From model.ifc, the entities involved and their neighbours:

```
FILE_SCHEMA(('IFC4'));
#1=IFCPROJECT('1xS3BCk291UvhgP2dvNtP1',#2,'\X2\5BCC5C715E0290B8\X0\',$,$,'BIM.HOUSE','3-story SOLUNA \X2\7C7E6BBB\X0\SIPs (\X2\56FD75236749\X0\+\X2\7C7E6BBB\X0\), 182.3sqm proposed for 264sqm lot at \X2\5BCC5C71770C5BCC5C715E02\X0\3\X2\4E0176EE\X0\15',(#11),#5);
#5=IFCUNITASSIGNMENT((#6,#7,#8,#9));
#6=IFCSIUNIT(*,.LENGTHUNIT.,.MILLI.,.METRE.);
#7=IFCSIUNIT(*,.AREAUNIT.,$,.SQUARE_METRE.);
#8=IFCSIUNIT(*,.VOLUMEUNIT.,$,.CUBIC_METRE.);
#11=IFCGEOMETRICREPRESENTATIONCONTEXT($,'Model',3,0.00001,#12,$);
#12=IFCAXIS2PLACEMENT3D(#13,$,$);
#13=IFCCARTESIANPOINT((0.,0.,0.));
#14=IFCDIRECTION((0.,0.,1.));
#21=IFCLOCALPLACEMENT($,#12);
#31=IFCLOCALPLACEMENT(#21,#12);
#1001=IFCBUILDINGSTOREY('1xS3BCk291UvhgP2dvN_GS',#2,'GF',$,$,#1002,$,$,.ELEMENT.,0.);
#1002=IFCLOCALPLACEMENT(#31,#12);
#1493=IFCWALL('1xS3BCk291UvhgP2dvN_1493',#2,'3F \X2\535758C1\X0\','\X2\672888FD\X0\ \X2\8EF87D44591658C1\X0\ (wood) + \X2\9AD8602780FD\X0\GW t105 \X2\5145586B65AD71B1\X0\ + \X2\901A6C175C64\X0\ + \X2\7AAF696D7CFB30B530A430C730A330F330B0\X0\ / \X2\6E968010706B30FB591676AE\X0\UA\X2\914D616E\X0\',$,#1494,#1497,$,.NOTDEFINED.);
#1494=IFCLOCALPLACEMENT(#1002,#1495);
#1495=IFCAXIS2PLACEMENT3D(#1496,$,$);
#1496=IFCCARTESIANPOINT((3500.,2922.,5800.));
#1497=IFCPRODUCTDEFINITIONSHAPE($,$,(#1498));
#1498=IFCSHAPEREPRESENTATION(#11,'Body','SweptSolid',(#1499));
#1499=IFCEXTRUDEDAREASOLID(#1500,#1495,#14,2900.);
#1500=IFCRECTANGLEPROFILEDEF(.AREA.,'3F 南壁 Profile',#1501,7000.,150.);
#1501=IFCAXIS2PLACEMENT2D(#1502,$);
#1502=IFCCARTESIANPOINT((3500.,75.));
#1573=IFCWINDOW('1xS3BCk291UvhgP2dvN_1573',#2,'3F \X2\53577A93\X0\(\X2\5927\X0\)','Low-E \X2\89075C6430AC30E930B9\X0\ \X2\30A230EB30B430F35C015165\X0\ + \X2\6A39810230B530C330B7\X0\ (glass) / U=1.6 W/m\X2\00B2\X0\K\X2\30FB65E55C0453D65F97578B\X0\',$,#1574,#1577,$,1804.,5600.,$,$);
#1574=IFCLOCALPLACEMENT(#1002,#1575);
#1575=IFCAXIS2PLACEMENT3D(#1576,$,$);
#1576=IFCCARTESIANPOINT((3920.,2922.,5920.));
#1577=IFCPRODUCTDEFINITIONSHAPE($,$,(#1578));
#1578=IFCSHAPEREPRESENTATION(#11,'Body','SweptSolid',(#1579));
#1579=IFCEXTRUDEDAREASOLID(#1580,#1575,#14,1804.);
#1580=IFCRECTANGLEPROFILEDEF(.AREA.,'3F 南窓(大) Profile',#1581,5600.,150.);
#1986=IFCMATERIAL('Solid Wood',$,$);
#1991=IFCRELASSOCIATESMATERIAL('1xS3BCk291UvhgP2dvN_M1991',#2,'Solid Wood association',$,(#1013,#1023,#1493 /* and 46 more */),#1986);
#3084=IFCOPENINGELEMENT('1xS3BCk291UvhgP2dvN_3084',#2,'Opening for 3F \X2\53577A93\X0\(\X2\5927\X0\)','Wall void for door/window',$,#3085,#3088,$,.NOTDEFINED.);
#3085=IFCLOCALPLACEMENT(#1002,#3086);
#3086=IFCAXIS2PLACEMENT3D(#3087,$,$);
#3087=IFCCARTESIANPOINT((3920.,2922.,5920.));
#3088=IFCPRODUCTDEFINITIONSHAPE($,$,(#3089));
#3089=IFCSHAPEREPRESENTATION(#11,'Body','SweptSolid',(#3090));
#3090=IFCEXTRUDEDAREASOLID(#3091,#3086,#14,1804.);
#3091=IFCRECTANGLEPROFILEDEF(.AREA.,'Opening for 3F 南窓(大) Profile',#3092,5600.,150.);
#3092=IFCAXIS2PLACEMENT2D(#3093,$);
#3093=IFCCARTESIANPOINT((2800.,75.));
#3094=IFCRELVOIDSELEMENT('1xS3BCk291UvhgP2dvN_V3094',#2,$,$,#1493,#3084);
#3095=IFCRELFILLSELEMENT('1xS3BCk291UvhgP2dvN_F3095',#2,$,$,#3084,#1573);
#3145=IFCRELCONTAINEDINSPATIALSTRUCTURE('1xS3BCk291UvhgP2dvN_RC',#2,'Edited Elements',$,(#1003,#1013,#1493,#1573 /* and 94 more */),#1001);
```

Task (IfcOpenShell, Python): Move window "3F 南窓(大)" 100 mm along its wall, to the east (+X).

```python
import ifcopenshell
import ifcopenshell.api.geometry
import ifcopenshell.util.placement
import ifcopenshell.util.unit

model = ifcopenshell.open("model.ifc")
unit_scale = ifcopenshell.util.unit.calculate_unit_scale(model)

window = model.by_id(1573)
opening = window.FillsVoids[0].RelatingOpeningElement
wall = opening.VoidsElements[0].RelatingBuildingElement

wall_matrix = ifcopenshell.util.placement.get_local_placement(wall.ObjectPlacement)
shift = wall_matrix[:3, 0] * 0.1 / unit_scale
before = ifcopenshell.util.placement.get_local_placement(window.ObjectPlacement)[:3, 3].copy()

# The window is not placed relative to its opening, so move both.
for product in (opening, window):
    matrix = ifcopenshell.util.placement.get_local_placement(product.ObjectPlacement)
    matrix[:3, 3] += shift
    ifcopenshell.api.geometry.edit_object_placement(model, product=product, matrix=matrix, is_si=False)

after = ifcopenshell.util.placement.get_local_placement(window.ObjectPlacement)[:3, 3]
print("window moved by", (after - before).round(3) + 0.0)

model.write("model-out.ifc")
```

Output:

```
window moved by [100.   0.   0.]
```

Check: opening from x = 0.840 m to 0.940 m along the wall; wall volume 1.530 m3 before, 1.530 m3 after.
